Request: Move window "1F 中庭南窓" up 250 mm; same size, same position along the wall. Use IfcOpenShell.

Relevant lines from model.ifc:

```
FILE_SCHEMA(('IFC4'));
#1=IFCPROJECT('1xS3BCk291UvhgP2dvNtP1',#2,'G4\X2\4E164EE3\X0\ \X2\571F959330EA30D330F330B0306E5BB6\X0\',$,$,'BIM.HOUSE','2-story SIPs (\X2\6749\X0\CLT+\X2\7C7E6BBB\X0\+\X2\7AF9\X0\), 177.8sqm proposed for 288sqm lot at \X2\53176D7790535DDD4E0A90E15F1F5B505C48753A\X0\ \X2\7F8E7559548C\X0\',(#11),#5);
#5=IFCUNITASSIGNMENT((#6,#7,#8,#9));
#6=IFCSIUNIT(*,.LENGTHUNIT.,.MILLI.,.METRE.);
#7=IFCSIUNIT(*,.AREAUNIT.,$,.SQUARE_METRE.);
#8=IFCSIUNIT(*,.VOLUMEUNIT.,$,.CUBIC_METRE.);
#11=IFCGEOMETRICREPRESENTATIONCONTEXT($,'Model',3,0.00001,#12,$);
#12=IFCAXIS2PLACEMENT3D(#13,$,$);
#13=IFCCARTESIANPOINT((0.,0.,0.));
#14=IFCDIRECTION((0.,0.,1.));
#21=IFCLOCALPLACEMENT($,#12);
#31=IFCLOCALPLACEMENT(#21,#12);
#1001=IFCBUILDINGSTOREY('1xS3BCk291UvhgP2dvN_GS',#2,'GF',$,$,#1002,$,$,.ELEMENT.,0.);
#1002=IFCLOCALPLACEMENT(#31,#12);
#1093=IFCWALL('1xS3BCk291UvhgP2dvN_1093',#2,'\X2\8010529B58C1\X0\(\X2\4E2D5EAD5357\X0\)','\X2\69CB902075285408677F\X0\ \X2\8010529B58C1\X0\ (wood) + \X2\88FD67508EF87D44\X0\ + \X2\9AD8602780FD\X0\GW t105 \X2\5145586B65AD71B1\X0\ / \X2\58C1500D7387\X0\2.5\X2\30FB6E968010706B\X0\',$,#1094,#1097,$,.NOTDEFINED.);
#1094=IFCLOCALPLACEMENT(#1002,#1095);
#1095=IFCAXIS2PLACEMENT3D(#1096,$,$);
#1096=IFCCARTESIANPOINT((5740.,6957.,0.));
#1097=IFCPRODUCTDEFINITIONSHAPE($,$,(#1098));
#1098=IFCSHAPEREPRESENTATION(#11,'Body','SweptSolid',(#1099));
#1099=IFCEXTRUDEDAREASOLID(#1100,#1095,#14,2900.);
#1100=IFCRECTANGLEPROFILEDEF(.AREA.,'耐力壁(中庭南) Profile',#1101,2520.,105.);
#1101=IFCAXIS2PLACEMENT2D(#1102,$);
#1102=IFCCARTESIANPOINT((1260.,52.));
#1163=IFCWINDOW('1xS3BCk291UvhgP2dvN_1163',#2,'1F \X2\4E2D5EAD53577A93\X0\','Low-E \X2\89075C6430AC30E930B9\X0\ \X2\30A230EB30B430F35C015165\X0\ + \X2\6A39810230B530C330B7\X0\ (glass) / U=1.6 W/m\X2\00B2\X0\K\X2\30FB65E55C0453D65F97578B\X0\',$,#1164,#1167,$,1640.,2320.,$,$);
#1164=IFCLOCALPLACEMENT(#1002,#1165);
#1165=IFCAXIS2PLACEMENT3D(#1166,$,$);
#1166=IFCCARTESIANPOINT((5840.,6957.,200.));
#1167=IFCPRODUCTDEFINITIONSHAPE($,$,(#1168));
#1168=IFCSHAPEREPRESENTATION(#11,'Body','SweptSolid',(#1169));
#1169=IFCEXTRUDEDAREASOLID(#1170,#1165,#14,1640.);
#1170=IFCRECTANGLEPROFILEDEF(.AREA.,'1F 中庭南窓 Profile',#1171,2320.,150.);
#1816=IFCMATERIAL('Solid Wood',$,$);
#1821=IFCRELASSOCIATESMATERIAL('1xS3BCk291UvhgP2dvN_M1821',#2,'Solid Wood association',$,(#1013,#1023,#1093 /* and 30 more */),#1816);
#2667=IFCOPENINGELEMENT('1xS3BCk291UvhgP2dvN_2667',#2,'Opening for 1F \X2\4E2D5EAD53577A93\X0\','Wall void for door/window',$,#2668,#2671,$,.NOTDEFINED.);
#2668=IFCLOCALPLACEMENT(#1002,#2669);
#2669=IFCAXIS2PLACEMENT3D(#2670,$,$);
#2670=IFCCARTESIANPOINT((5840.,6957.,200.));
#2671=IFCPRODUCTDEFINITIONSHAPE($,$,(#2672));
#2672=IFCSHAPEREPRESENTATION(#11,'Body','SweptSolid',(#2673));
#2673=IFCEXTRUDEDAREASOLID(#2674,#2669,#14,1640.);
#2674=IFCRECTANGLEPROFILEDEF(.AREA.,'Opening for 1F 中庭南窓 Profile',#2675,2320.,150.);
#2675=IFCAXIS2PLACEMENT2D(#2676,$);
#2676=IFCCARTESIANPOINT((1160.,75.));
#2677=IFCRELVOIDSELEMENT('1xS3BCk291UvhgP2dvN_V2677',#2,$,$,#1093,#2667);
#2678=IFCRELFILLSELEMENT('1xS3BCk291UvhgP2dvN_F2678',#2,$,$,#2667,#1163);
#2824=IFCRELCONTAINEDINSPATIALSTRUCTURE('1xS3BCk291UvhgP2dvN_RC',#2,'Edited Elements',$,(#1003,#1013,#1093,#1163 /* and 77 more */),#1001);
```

```python
import numpy as np
import ifcopenshell
import ifcopenshell.api.geometry
import ifcopenshell.util.placement
import ifcopenshell.util.unit

model = ifcopenshell.open("model.ifc")
unit_scale = ifcopenshell.util.unit.calculate_unit_scale(model)

window = model.by_guid("1xS3BCk291UvhgP2dvN_1163")
opening = window.FillsVoids[0].RelatingOpeningElement
dz = 250.0

shift = np.array([0.0, 0.0, dz])
# The window is not placed relative to its opening, so move both.
for product in (opening, window):
    matrix = ifcopenshell.util.placement.get_local_placement(product.ObjectPlacement)
    matrix[:3, 3] += shift
    ifcopenshell.api.geometry.edit_object_placement(model, product=product, matrix=matrix, is_si=False)

print(f"moved by {dz * unit_scale:+.3f} m")

model.write("model_rev.ifc")
```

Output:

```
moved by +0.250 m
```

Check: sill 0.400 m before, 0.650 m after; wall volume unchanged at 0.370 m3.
